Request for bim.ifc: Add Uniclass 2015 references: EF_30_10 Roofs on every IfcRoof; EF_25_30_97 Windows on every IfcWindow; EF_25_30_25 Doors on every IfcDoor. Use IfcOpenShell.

First a look at what the model holds.

```python
import ifcopenshell

model = ifcopenshell.open("bim.ifc")
print(model.schema)
print("classifications:", [c.Name for c in model.by_type("IfcClassification")])
for ifc_class in ("IfcDoor", "IfcRoof", "IfcStair", "IfcWall", "IfcWindow"):
    print(ifc_class, len(model.by_type(ifc_class)))
```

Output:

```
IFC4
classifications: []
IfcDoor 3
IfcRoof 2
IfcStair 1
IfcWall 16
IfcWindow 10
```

```python
import ifcopenshell
import ifcopenshell.api.classification

model = ifcopenshell.open("bim.ifc")

system = ifcopenshell.api.classification.add_classification(model, classification="Uniclass 2015")

codes = {
    "IfcRoof": ("EF_30_10", "Roofs"),
    "IfcWindow": ("EF_25_30_97", "Windows"),
    "IfcDoor": ("EF_25_30_25", "Doors"),
}
for ifc_class, (code, name) in codes.items():
    products = model.by_type(ifc_class)
    ifcopenshell.api.classification.add_reference(
        model, products=products, classification=system, identification=code, name=name
    )
    print(code, len(products))

model.write("bim_edited.ifc")
```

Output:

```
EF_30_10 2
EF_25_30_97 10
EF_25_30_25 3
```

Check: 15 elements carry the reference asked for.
